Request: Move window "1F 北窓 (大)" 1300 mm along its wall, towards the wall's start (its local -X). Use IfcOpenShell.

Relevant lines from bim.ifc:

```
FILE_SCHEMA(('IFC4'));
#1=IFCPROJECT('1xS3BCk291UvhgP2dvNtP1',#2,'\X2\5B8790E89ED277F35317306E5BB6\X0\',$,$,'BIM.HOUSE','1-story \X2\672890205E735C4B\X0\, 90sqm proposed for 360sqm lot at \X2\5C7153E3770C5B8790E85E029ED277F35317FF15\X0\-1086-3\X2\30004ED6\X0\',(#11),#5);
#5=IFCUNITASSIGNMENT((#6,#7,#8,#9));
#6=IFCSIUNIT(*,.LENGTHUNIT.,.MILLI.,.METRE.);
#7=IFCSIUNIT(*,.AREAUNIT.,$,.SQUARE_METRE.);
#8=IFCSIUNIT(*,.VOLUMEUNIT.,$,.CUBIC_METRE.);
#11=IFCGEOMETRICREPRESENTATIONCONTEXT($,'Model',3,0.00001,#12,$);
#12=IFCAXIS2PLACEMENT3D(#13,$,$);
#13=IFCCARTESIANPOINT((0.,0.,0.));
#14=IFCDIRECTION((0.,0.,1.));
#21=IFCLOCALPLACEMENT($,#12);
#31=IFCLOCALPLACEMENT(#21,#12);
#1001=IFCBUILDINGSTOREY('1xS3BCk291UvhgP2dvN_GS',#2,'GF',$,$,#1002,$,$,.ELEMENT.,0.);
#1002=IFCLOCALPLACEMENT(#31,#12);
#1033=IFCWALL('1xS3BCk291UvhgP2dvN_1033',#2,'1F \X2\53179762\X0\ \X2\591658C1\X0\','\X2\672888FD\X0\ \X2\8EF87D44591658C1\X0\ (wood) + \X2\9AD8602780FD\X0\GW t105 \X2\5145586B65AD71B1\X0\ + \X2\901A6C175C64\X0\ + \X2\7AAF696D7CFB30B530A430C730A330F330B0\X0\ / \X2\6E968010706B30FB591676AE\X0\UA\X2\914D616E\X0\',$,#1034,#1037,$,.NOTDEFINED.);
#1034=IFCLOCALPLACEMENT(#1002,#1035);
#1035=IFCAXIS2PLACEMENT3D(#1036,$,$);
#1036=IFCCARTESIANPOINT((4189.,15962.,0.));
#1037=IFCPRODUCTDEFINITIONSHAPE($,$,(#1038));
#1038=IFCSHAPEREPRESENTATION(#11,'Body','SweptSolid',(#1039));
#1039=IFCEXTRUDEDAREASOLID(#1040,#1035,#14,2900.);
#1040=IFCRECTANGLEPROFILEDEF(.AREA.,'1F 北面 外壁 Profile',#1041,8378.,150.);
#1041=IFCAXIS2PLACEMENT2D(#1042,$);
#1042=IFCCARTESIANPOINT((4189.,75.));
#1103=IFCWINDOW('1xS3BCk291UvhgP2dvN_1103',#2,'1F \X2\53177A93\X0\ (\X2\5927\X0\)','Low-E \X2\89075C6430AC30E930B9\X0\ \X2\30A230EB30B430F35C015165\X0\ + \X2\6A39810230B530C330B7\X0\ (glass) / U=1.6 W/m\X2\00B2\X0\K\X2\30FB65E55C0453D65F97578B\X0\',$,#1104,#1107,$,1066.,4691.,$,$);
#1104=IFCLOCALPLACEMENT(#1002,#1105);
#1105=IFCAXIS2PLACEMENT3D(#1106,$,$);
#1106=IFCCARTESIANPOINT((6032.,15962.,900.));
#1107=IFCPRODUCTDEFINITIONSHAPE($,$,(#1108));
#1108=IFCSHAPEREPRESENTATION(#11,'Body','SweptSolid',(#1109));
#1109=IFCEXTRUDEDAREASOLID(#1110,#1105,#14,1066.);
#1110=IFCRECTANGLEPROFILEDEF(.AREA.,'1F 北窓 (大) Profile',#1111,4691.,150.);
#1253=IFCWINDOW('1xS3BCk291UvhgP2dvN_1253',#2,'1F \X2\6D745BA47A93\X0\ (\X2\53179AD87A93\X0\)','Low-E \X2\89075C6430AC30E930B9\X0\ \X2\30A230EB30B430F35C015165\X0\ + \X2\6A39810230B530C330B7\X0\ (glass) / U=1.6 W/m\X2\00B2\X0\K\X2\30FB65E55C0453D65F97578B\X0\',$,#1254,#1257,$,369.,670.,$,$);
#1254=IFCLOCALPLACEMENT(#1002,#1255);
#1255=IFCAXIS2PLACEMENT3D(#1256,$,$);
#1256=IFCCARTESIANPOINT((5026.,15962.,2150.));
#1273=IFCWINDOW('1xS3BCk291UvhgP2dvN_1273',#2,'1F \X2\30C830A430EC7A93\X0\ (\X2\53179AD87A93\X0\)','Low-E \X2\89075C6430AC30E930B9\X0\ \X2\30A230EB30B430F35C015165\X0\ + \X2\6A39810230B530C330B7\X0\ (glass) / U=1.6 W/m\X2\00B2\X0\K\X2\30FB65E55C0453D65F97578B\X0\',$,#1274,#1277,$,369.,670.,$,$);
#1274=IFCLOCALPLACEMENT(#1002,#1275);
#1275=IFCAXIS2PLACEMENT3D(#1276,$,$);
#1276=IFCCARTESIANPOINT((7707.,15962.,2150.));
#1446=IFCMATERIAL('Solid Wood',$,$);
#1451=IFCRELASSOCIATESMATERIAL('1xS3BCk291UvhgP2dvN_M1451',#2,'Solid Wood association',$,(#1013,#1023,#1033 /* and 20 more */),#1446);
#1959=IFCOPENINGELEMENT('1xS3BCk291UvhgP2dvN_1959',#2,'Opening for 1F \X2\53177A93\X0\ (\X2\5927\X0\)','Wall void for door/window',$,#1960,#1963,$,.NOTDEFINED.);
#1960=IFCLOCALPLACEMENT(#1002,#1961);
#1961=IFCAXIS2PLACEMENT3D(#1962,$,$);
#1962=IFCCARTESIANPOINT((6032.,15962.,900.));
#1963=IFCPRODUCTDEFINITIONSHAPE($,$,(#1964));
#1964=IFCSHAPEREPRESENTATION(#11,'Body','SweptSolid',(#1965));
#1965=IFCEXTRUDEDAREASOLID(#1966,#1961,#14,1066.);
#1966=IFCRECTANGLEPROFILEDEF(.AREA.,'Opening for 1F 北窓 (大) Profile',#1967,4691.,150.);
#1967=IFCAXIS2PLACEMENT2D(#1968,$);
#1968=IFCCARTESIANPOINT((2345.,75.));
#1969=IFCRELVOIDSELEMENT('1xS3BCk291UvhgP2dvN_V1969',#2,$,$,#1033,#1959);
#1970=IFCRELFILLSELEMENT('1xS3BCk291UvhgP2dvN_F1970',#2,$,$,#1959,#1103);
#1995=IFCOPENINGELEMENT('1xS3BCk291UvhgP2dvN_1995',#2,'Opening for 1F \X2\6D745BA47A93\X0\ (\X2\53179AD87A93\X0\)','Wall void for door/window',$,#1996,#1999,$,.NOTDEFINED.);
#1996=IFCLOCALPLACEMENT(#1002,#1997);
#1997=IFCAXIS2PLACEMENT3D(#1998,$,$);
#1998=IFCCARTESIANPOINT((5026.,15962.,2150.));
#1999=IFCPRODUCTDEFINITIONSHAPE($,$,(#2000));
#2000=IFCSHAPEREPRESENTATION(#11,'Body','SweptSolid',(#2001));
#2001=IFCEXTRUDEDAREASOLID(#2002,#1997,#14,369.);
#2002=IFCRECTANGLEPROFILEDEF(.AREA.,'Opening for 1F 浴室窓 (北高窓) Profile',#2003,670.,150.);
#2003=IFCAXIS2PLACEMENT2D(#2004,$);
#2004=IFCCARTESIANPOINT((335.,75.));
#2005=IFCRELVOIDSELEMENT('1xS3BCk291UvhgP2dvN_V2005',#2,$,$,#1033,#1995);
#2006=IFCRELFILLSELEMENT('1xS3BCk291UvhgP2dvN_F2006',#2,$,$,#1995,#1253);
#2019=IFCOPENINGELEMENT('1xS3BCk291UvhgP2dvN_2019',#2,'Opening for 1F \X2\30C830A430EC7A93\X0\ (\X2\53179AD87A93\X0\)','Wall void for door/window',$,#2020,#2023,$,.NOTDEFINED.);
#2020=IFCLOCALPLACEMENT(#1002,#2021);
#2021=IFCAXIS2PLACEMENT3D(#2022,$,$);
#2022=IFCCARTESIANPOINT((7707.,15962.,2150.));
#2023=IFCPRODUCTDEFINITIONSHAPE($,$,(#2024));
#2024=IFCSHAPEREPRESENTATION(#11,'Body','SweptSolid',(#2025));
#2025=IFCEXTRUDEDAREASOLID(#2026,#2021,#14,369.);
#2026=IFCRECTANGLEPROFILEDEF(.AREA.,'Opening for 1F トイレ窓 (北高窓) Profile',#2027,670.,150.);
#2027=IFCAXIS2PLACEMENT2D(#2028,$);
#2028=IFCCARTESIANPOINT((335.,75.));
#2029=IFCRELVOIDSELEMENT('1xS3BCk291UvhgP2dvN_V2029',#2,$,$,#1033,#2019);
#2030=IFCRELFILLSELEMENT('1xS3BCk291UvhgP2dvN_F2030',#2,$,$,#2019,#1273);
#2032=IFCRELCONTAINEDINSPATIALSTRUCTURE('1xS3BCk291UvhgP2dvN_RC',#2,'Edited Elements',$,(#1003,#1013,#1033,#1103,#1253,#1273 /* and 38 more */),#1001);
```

```python
import ifcopenshell
import ifcopenshell.api.geometry
import ifcopenshell.util.placement

model = ifcopenshell.open("bim.ifc")

window = model.by_guid("1xS3BCk291UvhgP2dvN_1103")
opening = window.FillsVoids[0].RelatingOpeningElement
wall = opening.VoidsElements[0].RelatingBuildingElement

wall_matrix = ifcopenshell.util.placement.get_local_placement(wall.ObjectPlacement)
shift = wall_matrix[:3, 0] * -1300.0
before = ifcopenshell.util.placement.get_local_placement(window.ObjectPlacement)[:3, 3].copy()

# The window is not placed relative to its opening, so move both.
for product in (opening, window):
    matrix = ifcopenshell.util.placement.get_local_placement(product.ObjectPlacement)
    matrix[:3, 3] += shift
    ifcopenshell.api.geometry.edit_object_placement(model, product=product, matrix=matrix, is_si=False)

after = ifcopenshell.util.placement.get_local_placement(window.ObjectPlacement)[:3, 3]
print("window moved by", (after - before).round(3) + 0.0)

model.write("bim_edited.ifc")
```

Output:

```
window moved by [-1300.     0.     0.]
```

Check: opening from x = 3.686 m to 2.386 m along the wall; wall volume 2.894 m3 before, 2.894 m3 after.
